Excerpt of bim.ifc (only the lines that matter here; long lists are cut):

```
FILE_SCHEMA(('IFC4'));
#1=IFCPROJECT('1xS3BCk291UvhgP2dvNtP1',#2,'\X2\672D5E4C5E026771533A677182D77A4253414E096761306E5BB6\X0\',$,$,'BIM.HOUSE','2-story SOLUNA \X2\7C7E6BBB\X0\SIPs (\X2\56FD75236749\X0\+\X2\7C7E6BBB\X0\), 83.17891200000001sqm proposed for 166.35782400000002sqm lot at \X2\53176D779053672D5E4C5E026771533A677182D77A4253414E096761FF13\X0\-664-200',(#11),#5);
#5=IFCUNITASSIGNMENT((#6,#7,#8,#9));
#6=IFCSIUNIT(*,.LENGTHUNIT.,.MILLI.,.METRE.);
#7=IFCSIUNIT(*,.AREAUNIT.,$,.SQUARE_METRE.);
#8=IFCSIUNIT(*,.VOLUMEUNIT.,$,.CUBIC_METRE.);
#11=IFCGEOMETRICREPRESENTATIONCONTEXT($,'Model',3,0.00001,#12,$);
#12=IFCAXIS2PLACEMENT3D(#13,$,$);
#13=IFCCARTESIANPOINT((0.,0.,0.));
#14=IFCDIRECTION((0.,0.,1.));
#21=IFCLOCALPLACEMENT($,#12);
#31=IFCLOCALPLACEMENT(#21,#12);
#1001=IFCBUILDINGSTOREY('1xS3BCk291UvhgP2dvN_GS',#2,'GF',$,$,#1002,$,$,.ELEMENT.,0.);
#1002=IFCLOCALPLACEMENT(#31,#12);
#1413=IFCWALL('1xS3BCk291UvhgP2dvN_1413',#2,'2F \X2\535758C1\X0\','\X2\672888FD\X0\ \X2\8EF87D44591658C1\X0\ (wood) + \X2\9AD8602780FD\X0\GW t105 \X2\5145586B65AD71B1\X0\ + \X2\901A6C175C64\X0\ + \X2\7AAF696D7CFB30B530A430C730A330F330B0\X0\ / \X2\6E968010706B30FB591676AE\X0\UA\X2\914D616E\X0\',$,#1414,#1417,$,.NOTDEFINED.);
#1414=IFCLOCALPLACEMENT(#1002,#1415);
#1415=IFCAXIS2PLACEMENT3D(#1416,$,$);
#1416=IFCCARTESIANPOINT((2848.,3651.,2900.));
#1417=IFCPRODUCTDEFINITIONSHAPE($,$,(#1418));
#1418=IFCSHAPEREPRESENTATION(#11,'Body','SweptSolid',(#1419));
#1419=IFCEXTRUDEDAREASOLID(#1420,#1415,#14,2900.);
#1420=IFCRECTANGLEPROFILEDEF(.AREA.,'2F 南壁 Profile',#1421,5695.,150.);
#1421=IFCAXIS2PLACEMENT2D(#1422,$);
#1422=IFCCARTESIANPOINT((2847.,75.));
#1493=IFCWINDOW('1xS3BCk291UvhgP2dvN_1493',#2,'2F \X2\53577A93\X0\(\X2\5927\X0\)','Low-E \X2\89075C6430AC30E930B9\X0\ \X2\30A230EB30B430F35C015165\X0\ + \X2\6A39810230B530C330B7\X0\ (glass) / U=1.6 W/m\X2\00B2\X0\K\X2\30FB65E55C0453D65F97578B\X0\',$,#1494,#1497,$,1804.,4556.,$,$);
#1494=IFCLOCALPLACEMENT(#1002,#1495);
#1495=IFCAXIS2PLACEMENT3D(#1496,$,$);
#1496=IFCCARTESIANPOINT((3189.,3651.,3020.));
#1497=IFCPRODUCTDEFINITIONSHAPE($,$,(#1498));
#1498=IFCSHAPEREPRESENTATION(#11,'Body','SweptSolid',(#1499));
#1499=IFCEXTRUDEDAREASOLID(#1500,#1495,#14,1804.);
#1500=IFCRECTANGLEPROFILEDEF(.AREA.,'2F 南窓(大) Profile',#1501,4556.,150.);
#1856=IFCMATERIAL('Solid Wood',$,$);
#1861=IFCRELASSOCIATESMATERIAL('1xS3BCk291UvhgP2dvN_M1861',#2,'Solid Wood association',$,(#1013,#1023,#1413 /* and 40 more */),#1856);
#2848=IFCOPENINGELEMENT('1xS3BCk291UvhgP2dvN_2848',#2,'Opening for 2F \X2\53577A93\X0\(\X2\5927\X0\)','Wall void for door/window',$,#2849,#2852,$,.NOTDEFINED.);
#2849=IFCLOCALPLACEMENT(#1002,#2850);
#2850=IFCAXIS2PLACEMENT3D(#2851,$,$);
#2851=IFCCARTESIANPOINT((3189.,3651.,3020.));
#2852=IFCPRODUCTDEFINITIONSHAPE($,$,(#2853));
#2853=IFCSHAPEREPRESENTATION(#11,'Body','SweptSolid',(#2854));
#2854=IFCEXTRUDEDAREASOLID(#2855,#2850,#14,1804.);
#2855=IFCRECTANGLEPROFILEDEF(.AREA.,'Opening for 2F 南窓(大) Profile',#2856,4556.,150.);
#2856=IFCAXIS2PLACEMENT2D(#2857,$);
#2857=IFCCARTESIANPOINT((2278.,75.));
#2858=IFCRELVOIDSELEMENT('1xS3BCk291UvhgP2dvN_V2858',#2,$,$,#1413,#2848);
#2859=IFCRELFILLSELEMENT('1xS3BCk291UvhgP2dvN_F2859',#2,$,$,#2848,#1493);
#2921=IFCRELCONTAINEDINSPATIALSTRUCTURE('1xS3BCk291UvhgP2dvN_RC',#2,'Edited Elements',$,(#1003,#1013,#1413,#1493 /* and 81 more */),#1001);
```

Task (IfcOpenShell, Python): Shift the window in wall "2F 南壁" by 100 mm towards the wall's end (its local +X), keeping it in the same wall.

```python
import ifcopenshell
import ifcopenshell.api.geometry
import ifcopenshell.util.placement
import ifcopenshell.util.unit

model = ifcopenshell.open("bim.ifc")
unit_scale = ifcopenshell.util.unit.calculate_unit_scale(model)

window = model.by_guid("1xS3BCk291UvhgP2dvN_1493")
opening = window.FillsVoids[0].RelatingOpeningElement
wall = opening.VoidsElements[0].RelatingBuildingElement

wall_matrix = ifcopenshell.util.placement.get_local_placement(wall.ObjectPlacement)
shift = wall_matrix[:3, 0] * 0.1 / unit_scale
before = ifcopenshell.util.placement.get_local_placement(window.ObjectPlacement)[:3, 3].copy()

# The window is not placed relative to its opening, so move both.
for product in (opening, window):
    matrix = ifcopenshell.util.placement.get_local_placement(product.ObjectPlacement)
    matrix[:3, 3] += shift
    ifcopenshell.api.geometry.edit_object_placement(model, product=product, matrix=matrix, is_si=False)

after = ifcopenshell.util.placement.get_local_placement(window.ObjectPlacement)[:3, 3]
print("window moved by", (after - before).round(3) + 0.0)

model.write("bim-out.ifc")
```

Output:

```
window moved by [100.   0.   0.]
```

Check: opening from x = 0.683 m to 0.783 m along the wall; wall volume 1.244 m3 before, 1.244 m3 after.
